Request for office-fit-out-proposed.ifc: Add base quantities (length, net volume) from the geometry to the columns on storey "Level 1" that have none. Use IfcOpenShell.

First a look at what the model holds.

```python
import ifcopenshell
import ifcopenshell.util.element
import ifcopenshell.util.unit

model = ifcopenshell.open("office-fit-out-proposed.ifc")
print(model.schema)
for unit_type in ("LENGTHUNIT", "AREAUNIT", "VOLUMEUNIT"):
    print(unit_type, ifcopenshell.util.unit.calculate_unit_scale(model, unit_type))
storey = next(s for s in model.by_type("IfcBuildingStorey") if s.Name == "Level 1")
columns = [e for e in ifcopenshell.util.element.get_decomposition(storey) if e.is_a("IfcColumn")]
for e in sorted(columns, key=lambda e: e.id()):
    print(e.id(), e.is_a(), e.Name, list(ifcopenshell.util.element.get_psets(e, qtos_only=True)), sep=" | ")
```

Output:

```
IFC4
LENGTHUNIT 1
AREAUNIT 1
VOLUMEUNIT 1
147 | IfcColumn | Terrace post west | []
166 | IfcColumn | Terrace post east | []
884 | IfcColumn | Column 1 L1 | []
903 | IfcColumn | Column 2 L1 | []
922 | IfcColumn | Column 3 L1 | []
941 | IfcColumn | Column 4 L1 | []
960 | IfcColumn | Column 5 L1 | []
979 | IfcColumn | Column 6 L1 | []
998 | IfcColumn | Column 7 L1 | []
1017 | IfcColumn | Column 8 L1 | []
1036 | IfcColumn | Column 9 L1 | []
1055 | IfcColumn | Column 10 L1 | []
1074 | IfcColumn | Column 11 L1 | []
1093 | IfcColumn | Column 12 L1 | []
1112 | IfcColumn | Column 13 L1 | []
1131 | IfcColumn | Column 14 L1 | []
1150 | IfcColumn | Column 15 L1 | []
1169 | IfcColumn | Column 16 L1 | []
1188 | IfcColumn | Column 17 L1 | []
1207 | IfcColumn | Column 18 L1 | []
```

```python
import ifcopenshell
import ifcopenshell.api.pset
import ifcopenshell.geom
import ifcopenshell.util.element
import ifcopenshell.util.shape
import ifcopenshell.util.unit

model = ifcopenshell.open("office-fit-out-proposed.ifc")
unit_scale = ifcopenshell.util.unit.calculate_unit_scale(model)
volume_scale = ifcopenshell.util.unit.calculate_unit_scale(model, "VOLUMEUNIT")
settings = ifcopenshell.geom.settings()

storey = next(s for s in model.by_type("IfcBuildingStorey") if s.Name == "Level 1")
columns = [e for e in ifcopenshell.util.element.get_decomposition(storey) if e.is_a("IfcColumn")]

for e in sorted(columns, key=lambda e: e.id()):
    if ifcopenshell.util.element.get_psets(e, qtos_only=True, should_inherit=False):
        continue
    # Geometry comes back in metres, in the element's own axes.
    shape = ifcopenshell.geom.create_shape(settings, e)
    values = {
        "Length": ifcopenshell.util.shape.get_z(shape.geometry) / unit_scale,
        "NetVolume": ifcopenshell.util.shape.get_volume(shape.geometry) / volume_scale,
    }
    qto = ifcopenshell.api.pset.add_qto(model, product=e, name="Qto_ColumnBaseQuantities")
    ifcopenshell.api.pset.edit_qto(model, qto=qto, properties=values)
    print(e.id(), {k: round(v, 3) for k, v in values.items()})

model.write("office-fit-out-proposed_v2.ifc")
```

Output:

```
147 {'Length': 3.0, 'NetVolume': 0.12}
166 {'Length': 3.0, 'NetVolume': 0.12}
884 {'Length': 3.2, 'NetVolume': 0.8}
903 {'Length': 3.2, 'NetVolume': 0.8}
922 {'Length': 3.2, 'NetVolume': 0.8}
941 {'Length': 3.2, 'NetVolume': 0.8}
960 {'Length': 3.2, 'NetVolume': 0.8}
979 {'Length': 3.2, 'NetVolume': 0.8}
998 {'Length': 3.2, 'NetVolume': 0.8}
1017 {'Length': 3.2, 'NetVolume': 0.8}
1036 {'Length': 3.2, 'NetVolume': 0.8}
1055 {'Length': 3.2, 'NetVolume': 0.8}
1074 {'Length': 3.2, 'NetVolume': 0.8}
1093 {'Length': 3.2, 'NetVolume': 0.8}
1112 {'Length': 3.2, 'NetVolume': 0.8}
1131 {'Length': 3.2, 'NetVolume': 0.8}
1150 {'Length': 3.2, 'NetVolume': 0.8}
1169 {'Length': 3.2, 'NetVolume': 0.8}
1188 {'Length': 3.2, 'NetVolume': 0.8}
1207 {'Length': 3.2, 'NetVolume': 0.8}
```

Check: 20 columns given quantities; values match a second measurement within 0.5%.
